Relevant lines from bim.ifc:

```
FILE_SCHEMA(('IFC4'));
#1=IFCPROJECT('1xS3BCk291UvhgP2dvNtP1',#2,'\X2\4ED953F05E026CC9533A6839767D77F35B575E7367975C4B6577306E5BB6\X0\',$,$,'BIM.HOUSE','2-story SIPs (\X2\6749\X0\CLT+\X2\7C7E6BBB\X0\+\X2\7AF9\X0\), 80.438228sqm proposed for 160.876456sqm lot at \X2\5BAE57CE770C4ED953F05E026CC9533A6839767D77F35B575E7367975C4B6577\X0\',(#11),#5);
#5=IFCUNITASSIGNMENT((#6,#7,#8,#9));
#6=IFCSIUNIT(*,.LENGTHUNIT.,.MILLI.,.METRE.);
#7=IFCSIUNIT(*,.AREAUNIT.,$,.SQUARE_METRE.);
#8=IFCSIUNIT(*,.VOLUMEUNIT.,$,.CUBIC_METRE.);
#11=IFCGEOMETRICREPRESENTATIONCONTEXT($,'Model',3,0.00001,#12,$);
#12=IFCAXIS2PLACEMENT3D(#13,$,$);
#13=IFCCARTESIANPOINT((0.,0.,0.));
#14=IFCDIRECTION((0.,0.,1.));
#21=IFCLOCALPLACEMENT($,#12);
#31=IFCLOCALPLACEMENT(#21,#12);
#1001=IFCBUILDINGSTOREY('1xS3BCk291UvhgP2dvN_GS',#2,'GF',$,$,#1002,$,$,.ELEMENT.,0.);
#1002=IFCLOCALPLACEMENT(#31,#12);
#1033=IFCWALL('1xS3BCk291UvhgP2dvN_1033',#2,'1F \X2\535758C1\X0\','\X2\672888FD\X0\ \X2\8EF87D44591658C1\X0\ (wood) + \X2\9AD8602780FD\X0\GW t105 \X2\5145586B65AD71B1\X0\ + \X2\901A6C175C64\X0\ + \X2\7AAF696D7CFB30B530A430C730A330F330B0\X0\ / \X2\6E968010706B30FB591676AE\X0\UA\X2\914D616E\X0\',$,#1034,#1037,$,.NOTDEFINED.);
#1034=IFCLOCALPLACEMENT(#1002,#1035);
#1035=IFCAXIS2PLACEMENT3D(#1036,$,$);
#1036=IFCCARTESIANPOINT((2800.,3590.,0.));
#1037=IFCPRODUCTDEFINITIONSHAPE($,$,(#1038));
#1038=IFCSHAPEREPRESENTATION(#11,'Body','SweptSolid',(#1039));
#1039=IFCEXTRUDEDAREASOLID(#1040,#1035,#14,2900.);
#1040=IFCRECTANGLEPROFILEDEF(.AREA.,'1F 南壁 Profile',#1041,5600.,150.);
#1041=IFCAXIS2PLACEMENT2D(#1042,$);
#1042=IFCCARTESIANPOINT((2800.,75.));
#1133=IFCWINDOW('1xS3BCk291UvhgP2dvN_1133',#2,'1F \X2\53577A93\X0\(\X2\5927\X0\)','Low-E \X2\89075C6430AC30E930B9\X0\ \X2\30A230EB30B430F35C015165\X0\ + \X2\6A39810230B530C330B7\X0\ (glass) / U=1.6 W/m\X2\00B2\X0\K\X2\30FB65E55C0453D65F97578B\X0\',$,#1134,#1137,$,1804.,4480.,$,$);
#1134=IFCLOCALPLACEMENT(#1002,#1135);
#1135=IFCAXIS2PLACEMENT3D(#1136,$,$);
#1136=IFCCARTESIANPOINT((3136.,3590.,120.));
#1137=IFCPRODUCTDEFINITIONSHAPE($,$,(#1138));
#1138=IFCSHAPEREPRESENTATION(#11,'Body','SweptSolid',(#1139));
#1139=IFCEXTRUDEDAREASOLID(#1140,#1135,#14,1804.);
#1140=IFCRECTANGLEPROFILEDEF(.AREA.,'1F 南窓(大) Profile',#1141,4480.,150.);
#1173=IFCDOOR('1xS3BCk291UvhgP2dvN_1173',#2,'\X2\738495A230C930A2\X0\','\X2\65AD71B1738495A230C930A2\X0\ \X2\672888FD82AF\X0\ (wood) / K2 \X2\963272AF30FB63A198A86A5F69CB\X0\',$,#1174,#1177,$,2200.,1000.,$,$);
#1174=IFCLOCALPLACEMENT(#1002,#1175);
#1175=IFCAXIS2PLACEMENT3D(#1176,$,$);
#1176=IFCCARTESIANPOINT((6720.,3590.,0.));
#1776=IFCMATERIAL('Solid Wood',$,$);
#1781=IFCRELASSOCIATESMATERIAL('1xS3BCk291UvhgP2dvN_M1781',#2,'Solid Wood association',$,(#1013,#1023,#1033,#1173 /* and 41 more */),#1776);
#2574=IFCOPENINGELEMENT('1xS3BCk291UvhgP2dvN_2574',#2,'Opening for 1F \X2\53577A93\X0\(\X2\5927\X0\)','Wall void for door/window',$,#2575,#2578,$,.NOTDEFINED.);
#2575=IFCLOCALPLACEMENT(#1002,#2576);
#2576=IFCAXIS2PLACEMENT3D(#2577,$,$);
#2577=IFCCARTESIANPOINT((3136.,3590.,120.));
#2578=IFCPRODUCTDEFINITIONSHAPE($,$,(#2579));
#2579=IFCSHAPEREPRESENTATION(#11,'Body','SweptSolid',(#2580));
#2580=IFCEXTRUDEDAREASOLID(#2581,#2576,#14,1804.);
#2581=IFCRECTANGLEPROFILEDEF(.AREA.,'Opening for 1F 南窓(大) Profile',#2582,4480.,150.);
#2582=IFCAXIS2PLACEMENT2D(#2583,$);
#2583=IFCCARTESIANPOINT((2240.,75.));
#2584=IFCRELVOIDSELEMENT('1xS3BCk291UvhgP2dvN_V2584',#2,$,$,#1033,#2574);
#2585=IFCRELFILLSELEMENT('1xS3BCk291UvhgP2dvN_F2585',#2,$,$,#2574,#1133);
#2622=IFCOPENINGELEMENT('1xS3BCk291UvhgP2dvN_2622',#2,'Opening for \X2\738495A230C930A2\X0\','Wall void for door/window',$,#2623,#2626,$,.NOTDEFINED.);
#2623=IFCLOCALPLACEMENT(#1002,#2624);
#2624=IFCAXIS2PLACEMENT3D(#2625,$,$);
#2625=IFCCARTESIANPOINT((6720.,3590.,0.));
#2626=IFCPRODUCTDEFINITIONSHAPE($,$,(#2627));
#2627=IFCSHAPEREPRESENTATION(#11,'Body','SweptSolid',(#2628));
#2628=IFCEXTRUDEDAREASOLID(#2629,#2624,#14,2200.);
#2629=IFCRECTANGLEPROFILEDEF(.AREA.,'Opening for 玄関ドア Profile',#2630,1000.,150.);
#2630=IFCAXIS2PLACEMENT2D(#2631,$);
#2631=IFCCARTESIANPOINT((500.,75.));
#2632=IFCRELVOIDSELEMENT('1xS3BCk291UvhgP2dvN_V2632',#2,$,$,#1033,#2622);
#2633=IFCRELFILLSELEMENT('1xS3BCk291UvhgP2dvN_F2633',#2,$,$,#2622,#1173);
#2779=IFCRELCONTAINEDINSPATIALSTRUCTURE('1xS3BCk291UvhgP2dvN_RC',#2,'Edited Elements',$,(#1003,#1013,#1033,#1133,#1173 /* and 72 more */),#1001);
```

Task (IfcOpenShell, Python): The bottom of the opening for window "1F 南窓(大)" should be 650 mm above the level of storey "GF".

```python
import numpy as np
import ifcopenshell
import ifcopenshell.api.geometry
import ifcopenshell.geom
import ifcopenshell.util.element
import ifcopenshell.util.placement
import ifcopenshell.util.shape
import ifcopenshell.util.unit

model = ifcopenshell.open("bim.ifc")
unit_scale = ifcopenshell.util.unit.calculate_unit_scale(model)

window = model.by_guid("1xS3BCk291UvhgP2dvN_1133")
opening = window.FillsVoids[0].RelatingOpeningElement
storey = ifcopenshell.util.element.get_container(window, ifc_class="IfcBuildingStorey")
level = ifcopenshell.util.placement.get_local_placement(storey.ObjectPlacement)[2, 3]

# The opening's origin need not be at the sill, so measure its lowest point.
shape = ifcopenshell.geom.create_shape(ifcopenshell.geom.settings(), opening)
bottom = ifcopenshell.util.shape.get_shape_bottom_elevation(shape, shape.geometry) / unit_scale
dz = level + 0.65 / unit_scale - bottom

shift = np.array([0.0, 0.0, dz])
# The window is not placed relative to its opening, so move both.
for product in (opening, window):
    matrix = ifcopenshell.util.placement.get_local_placement(product.ObjectPlacement)
    matrix[:3, 3] += shift
    ifcopenshell.api.geometry.edit_object_placement(model, product=product, matrix=matrix, is_si=False)

print(f"moved by {dz * unit_scale:+.3f} m")

model.write("bim_rev.ifc")
```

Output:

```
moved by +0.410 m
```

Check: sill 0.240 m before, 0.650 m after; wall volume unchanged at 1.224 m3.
